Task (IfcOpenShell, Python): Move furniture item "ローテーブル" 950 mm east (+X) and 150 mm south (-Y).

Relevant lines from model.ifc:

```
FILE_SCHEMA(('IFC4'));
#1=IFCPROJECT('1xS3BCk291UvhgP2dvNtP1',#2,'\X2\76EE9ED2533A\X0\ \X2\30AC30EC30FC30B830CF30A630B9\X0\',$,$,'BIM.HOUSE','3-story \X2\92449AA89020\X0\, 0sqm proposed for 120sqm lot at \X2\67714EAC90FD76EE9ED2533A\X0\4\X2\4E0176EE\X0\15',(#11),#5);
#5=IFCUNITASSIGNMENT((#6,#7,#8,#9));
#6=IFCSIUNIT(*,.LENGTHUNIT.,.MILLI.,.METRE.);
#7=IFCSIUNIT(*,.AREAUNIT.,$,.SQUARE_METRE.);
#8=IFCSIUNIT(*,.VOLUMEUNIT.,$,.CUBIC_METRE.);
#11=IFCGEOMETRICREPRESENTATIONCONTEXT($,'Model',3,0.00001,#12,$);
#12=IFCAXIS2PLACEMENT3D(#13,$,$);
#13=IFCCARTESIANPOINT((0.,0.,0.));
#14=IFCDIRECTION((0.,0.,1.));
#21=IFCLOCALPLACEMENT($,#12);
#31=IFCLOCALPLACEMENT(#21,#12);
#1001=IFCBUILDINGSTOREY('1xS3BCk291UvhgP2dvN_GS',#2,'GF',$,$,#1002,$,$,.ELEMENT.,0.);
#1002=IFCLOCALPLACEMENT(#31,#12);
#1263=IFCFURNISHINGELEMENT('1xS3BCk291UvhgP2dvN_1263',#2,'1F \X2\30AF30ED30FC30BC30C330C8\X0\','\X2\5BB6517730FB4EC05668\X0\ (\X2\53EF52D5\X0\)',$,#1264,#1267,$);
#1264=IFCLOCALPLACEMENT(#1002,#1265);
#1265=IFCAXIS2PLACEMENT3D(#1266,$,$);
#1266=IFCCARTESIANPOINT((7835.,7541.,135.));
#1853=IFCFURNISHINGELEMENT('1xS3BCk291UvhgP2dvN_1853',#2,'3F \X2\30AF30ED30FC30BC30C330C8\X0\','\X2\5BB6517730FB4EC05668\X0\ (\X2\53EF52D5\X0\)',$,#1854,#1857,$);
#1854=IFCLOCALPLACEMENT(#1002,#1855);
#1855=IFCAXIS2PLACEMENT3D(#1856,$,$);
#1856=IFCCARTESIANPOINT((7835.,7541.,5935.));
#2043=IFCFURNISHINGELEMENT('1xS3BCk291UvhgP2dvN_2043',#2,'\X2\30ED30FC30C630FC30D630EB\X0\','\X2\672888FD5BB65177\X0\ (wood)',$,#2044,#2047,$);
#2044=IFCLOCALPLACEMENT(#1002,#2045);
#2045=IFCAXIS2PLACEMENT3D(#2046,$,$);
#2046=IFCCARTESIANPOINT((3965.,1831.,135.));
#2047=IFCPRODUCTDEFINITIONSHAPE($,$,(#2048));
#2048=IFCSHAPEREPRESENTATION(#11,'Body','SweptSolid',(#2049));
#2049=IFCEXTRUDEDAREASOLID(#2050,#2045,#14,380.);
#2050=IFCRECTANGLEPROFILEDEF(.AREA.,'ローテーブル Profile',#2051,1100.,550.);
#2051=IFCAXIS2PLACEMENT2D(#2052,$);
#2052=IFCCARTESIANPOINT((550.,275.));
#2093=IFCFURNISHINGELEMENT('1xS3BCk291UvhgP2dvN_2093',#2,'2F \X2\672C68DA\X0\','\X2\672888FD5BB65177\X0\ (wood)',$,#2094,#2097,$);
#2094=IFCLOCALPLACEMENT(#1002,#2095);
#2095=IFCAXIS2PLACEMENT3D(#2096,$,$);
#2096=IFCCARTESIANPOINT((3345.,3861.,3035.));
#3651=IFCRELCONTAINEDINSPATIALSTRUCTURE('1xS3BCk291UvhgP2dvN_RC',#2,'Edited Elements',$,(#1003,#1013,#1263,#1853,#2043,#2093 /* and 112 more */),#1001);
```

```python
import ifcopenshell
import ifcopenshell.api.geometry
import ifcopenshell.util.placement
import ifcopenshell.util.unit

model = ifcopenshell.open("model.ifc")
unit_scale = ifcopenshell.util.unit.calculate_unit_scale(model)

item = model.by_guid("1xS3BCk291UvhgP2dvN_2043")
matrix = ifcopenshell.util.placement.get_local_placement(item.ObjectPlacement)
matrix[0, 3] += 0.95 / unit_scale
matrix[1, 3] -= 0.15 / unit_scale
ifcopenshell.api.geometry.edit_object_placement(model, product=item, matrix=matrix, is_si=False)

print(ifcopenshell.util.placement.get_local_placement(item.ObjectPlacement).round(3) + 0.0)

model.write("model_updated.ifc")
```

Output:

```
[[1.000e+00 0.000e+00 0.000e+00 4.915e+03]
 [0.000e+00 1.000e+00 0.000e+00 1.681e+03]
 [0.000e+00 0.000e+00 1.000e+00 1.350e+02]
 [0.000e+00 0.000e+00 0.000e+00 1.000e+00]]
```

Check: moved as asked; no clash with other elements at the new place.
